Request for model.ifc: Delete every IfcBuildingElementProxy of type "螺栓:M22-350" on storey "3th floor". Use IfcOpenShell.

First a look at what the model holds.

```python
import ifcopenshell
import ifcopenshell.util.element

model = ifcopenshell.open("model.ifc")
print(model.schema)
storey = next(s for s in model.by_type("IfcBuildingStorey") if s.Name == "3th floor")
proxies = [e for e in ifcopenshell.util.element.get_decomposition(storey) if e.is_a("IfcBuildingElementProxy")]
seen = {}
for e in proxies:
    element_type = ifcopenshell.util.element.get_type(e)
    name = element_type.Name if element_type not in (None, e) else None
    seen[name] = seen.get(name, 0) + 1
for name, count in sorted(seen.items(), key=str):
    print(count, "x", name)
```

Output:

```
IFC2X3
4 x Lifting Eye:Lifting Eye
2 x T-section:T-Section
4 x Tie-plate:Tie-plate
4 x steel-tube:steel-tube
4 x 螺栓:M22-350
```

```python
import ifcopenshell
import ifcopenshell.api.root
import ifcopenshell.util.element

model = ifcopenshell.open("model.ifc")

storey = next(s for s in model.by_type("IfcBuildingStorey") if s.Name == "3th floor")
proxies = [e for e in ifcopenshell.util.element.get_decomposition(storey) if e.is_a("IfcBuildingElementProxy")]
targets = [e for e in proxies if (t := ifcopenshell.util.element.get_type(e)) not in (None, e) and t.Name == "螺栓:M22-350"]

for e in targets:
    ifcopenshell.api.root.remove_product(model, product=e)
print(len(targets), "removed")

model.write("model_rev.ifc")
```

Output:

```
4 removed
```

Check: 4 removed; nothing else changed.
